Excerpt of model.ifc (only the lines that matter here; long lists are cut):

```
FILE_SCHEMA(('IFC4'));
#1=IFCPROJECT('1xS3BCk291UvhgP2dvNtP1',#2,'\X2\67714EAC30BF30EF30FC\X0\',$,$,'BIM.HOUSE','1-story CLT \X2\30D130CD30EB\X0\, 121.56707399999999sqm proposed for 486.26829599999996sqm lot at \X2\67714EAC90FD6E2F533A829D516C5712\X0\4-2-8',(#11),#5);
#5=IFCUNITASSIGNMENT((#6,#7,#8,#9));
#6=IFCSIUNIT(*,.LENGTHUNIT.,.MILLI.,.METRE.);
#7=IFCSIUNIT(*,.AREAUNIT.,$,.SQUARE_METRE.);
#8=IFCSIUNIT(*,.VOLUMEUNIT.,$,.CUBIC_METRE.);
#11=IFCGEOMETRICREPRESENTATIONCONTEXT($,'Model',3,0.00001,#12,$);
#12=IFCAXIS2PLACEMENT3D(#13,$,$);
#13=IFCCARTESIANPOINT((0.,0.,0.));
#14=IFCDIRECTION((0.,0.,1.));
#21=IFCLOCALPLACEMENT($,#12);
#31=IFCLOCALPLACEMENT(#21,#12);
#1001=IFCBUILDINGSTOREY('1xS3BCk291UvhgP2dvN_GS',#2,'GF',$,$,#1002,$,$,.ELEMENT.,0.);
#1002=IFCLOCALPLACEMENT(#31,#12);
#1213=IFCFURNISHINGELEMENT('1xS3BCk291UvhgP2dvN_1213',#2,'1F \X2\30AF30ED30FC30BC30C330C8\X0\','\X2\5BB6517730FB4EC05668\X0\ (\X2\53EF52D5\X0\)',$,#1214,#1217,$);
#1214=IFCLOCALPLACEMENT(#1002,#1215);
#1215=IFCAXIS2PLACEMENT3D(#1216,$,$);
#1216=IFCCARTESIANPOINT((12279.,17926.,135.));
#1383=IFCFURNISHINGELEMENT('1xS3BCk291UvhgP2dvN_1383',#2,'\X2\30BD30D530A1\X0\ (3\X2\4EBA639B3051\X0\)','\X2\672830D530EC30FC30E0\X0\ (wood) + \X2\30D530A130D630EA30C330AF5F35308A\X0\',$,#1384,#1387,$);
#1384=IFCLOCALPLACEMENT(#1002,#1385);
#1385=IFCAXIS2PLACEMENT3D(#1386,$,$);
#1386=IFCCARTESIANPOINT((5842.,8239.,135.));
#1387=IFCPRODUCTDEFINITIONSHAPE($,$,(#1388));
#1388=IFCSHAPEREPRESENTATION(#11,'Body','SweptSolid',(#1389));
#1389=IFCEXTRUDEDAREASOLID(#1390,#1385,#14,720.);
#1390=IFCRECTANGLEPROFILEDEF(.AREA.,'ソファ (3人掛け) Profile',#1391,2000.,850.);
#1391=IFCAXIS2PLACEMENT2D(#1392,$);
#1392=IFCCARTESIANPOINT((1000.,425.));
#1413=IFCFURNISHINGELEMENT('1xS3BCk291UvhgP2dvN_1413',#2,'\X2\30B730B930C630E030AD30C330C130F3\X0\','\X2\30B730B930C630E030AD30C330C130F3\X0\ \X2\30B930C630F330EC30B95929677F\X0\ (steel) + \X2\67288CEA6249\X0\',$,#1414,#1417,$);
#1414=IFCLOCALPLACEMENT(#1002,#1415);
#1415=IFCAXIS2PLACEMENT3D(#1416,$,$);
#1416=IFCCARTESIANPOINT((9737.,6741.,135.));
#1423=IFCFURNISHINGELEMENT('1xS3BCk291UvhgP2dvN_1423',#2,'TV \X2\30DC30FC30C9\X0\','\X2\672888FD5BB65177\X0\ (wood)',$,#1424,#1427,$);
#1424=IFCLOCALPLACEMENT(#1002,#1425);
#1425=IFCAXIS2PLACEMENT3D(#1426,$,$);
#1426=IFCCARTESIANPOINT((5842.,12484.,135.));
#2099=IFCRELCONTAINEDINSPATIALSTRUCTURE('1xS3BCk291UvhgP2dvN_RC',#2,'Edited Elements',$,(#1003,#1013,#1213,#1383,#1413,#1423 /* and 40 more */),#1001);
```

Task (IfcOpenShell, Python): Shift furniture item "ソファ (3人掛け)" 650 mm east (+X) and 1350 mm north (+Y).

```python
import ifcopenshell
import ifcopenshell.api.geometry
import ifcopenshell.util.placement
import ifcopenshell.util.unit

model = ifcopenshell.open("model.ifc")
unit_scale = ifcopenshell.util.unit.calculate_unit_scale(model)

item = model.by_guid("1xS3BCk291UvhgP2dvN_1383")
matrix = ifcopenshell.util.placement.get_local_placement(item.ObjectPlacement)
matrix[0, 3] += 0.65 / unit_scale
matrix[1, 3] += 1.35 / unit_scale
ifcopenshell.api.geometry.edit_object_placement(model, product=item, matrix=matrix, is_si=False)

print(ifcopenshell.util.placement.get_local_placement(item.ObjectPlacement).round(3) + 0.0)

model.write("model_updated.ifc")
```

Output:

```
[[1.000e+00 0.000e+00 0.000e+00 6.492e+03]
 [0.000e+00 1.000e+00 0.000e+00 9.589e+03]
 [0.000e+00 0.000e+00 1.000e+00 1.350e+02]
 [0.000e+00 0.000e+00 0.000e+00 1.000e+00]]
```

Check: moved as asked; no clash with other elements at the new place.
